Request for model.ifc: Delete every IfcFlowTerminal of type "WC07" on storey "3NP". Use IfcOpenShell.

First a look at what the model holds.

```python
import ifcopenshell
import ifcopenshell.util.element

model = ifcopenshell.open("model.ifc")
print(model.schema)
storey = next(s for s in model.by_type("IfcBuildingStorey") if s.Name == "3NP")
terminals = [e for e in ifcopenshell.util.element.get_decomposition(storey) if e.is_a("IfcFlowTerminal")]
seen = {}
for e in terminals:
    element_type = ifcopenshell.util.element.get_type(e)
    name = element_type.Name if element_type not in (None, e) else None
    seen[name] = seen.get(name, 0) + 1
for name, count in sorted(seen.items(), key=str):
    print(count, "x", name)
```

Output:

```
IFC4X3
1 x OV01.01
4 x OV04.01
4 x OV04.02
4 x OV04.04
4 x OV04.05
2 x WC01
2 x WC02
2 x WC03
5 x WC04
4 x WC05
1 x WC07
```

```python
import ifcopenshell
import ifcopenshell.api.root
import ifcopenshell.util.element

model = ifcopenshell.open("model.ifc")

storey = next(s for s in model.by_type("IfcBuildingStorey") if s.Name == "3NP")
terminals = [e for e in ifcopenshell.util.element.get_decomposition(storey) if e.is_a("IfcFlowTerminal")]
targets = [e for e in terminals if (t := ifcopenshell.util.element.get_type(e)) not in (None, e) and t.Name == "WC07"]

for e in targets:
    ifcopenshell.api.root.remove_product(model, product=e)
print(len(targets), "removed")

model.write("model_updated.ifc")
```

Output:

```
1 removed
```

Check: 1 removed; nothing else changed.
